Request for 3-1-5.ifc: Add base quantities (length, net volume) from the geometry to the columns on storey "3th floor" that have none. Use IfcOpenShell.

First a look at what the model holds.

```python
import ifcopenshell
import ifcopenshell.util.element
import ifcopenshell.util.unit

model = ifcopenshell.open("3-1-5.ifc")
print(model.schema)
for unit_type in ("LENGTHUNIT", "AREAUNIT", "VOLUMEUNIT"):
    print(unit_type, ifcopenshell.util.unit.calculate_unit_scale(model, unit_type))
storey = next(s for s in model.by_type("IfcBuildingStorey") if s.Name == "3th floor")
columns = [e for e in ifcopenshell.util.element.get_decomposition(storey) if e.is_a("IfcColumn")]
for e in sorted(columns, key=lambda e: e.id()):
    print(e.id(), e.is_a(), e.Name, list(ifcopenshell.util.element.get_psets(e, qtos_only=True)), sep=" | ")
```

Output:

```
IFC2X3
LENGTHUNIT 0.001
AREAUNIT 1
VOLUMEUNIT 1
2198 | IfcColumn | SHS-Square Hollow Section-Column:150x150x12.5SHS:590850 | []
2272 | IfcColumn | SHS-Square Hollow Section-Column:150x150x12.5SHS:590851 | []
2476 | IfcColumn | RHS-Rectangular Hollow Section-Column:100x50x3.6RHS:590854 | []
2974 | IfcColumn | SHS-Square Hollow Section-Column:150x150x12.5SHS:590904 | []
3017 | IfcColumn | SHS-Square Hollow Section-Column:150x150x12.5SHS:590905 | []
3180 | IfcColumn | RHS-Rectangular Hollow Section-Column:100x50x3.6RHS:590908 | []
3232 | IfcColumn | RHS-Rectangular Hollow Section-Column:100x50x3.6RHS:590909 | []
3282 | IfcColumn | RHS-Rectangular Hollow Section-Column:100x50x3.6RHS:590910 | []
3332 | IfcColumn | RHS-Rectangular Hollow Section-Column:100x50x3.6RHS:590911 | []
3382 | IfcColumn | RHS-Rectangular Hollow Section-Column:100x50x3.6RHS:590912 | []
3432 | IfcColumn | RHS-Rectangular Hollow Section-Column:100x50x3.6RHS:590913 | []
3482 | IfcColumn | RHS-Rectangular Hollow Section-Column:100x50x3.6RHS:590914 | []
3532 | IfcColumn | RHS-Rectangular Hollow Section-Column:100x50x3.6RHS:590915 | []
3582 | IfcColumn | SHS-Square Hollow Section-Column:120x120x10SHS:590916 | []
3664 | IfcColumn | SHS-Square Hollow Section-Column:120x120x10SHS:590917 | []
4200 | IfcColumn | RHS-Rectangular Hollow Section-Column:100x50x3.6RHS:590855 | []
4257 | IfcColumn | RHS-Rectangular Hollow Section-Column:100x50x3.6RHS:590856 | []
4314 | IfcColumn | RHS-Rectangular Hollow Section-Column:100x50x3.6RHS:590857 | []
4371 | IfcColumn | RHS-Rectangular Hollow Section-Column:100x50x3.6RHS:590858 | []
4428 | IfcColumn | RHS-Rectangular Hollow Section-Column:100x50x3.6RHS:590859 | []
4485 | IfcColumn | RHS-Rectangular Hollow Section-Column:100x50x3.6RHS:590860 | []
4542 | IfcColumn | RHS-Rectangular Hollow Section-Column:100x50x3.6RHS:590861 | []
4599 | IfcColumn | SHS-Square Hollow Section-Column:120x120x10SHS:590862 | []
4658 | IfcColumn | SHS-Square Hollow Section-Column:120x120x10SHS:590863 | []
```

```python
import ifcopenshell
import ifcopenshell.api.pset
import ifcopenshell.geom
import ifcopenshell.util.element
import ifcopenshell.util.shape
import ifcopenshell.util.unit

model = ifcopenshell.open("3-1-5.ifc")
unit_scale = ifcopenshell.util.unit.calculate_unit_scale(model)
volume_scale = ifcopenshell.util.unit.calculate_unit_scale(model, "VOLUMEUNIT")
settings = ifcopenshell.geom.settings()

storey = next(s for s in model.by_type("IfcBuildingStorey") if s.Name == "3th floor")
columns = [e for e in ifcopenshell.util.element.get_decomposition(storey) if e.is_a("IfcColumn")]

for e in sorted(columns, key=lambda e: e.id()):
    if ifcopenshell.util.element.get_psets(e, qtos_only=True, should_inherit=False):
        continue
    # Geometry comes back in metres, in the element's own axes.
    shape = ifcopenshell.geom.create_shape(settings, e)
    values = {
        "Length": ifcopenshell.util.shape.get_z(shape.geometry) / unit_scale,
        "NetVolume": ifcopenshell.util.shape.get_volume(shape.geometry) / volume_scale,
    }
    qto = ifcopenshell.api.pset.add_qto(model, product=e, name="BaseQuantities")
    ifcopenshell.api.pset.edit_qto(model, qto=qto, properties=values)
    print(e.id(), {k: round(v, 3) for k, v in values.items()})

model.write("3-1-5-out.ifc")
```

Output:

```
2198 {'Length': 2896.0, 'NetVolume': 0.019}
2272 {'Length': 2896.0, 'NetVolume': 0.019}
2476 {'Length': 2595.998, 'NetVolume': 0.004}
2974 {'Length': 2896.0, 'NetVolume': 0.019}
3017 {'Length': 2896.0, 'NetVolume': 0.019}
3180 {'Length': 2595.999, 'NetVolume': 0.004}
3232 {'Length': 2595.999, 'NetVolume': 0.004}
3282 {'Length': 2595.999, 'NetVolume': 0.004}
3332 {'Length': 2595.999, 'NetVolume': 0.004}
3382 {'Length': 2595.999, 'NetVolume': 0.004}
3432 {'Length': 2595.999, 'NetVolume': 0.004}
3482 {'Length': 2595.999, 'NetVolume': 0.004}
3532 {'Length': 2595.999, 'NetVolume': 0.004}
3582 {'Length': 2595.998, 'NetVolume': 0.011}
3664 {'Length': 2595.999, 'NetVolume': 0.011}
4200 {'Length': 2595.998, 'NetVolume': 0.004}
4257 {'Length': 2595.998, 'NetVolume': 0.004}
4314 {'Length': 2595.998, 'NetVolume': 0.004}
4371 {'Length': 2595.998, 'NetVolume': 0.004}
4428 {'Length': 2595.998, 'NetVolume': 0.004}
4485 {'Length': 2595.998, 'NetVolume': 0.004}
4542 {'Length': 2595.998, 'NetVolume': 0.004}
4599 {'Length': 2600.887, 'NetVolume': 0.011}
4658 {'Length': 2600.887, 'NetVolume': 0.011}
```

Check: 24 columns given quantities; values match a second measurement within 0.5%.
